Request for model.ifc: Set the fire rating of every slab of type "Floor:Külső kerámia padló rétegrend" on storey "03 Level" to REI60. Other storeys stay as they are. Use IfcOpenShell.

First a look at what the model holds.

```python
import ifcopenshell
import ifcopenshell.util.element

model = ifcopenshell.open("model.ifc")
print(model.schema)
storey = next(s for s in model.by_type("IfcBuildingStorey") if s.Name == "03 Level")
slabs = [e for e in ifcopenshell.util.element.get_decomposition(storey) if e.is_a("IfcSlab")]
seen = {}
for e in slabs:
    element_type = ifcopenshell.util.element.get_type(e)
    key = (element_type.Name if element_type != e and element_type else None, ifcopenshell.util.element.get_pset(e, "Pset_SlabCommon", "FireRating"))
    seen[key] = seen.get(key, 0) + 1
for (name, value), count in sorted(seen.items(), key=str):
    print(count, "x", name, "|", value)
```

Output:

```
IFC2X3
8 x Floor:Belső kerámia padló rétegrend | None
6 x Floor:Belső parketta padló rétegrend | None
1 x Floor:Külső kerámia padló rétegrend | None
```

```python
import ifcopenshell
import ifcopenshell.api.pset
import ifcopenshell.util.element

model = ifcopenshell.open("model.ifc")

storey = next(s for s in model.by_type("IfcBuildingStorey") if s.Name == "03 Level")
slabs = [e for e in ifcopenshell.util.element.get_decomposition(storey) if e.is_a("IfcSlab")]

count = 0
for e in slabs:
    element_type = ifcopenshell.util.element.get_type(e)
    if element_type in (None, e) or element_type.Name != "Floor:Külső kerámia padló rétegrend":
        continue
    # add_pset returns the element's existing set when there is one.
    pset = ifcopenshell.api.pset.add_pset(model, product=e, name="Pset_SlabCommon")
    ifcopenshell.api.pset.edit_pset(model, pset=pset, properties={"FireRating": "REI60"})
    count += 1

print(count, "slabs updated")

model.write("model_v2.ifc")
```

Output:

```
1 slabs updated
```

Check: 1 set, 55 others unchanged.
